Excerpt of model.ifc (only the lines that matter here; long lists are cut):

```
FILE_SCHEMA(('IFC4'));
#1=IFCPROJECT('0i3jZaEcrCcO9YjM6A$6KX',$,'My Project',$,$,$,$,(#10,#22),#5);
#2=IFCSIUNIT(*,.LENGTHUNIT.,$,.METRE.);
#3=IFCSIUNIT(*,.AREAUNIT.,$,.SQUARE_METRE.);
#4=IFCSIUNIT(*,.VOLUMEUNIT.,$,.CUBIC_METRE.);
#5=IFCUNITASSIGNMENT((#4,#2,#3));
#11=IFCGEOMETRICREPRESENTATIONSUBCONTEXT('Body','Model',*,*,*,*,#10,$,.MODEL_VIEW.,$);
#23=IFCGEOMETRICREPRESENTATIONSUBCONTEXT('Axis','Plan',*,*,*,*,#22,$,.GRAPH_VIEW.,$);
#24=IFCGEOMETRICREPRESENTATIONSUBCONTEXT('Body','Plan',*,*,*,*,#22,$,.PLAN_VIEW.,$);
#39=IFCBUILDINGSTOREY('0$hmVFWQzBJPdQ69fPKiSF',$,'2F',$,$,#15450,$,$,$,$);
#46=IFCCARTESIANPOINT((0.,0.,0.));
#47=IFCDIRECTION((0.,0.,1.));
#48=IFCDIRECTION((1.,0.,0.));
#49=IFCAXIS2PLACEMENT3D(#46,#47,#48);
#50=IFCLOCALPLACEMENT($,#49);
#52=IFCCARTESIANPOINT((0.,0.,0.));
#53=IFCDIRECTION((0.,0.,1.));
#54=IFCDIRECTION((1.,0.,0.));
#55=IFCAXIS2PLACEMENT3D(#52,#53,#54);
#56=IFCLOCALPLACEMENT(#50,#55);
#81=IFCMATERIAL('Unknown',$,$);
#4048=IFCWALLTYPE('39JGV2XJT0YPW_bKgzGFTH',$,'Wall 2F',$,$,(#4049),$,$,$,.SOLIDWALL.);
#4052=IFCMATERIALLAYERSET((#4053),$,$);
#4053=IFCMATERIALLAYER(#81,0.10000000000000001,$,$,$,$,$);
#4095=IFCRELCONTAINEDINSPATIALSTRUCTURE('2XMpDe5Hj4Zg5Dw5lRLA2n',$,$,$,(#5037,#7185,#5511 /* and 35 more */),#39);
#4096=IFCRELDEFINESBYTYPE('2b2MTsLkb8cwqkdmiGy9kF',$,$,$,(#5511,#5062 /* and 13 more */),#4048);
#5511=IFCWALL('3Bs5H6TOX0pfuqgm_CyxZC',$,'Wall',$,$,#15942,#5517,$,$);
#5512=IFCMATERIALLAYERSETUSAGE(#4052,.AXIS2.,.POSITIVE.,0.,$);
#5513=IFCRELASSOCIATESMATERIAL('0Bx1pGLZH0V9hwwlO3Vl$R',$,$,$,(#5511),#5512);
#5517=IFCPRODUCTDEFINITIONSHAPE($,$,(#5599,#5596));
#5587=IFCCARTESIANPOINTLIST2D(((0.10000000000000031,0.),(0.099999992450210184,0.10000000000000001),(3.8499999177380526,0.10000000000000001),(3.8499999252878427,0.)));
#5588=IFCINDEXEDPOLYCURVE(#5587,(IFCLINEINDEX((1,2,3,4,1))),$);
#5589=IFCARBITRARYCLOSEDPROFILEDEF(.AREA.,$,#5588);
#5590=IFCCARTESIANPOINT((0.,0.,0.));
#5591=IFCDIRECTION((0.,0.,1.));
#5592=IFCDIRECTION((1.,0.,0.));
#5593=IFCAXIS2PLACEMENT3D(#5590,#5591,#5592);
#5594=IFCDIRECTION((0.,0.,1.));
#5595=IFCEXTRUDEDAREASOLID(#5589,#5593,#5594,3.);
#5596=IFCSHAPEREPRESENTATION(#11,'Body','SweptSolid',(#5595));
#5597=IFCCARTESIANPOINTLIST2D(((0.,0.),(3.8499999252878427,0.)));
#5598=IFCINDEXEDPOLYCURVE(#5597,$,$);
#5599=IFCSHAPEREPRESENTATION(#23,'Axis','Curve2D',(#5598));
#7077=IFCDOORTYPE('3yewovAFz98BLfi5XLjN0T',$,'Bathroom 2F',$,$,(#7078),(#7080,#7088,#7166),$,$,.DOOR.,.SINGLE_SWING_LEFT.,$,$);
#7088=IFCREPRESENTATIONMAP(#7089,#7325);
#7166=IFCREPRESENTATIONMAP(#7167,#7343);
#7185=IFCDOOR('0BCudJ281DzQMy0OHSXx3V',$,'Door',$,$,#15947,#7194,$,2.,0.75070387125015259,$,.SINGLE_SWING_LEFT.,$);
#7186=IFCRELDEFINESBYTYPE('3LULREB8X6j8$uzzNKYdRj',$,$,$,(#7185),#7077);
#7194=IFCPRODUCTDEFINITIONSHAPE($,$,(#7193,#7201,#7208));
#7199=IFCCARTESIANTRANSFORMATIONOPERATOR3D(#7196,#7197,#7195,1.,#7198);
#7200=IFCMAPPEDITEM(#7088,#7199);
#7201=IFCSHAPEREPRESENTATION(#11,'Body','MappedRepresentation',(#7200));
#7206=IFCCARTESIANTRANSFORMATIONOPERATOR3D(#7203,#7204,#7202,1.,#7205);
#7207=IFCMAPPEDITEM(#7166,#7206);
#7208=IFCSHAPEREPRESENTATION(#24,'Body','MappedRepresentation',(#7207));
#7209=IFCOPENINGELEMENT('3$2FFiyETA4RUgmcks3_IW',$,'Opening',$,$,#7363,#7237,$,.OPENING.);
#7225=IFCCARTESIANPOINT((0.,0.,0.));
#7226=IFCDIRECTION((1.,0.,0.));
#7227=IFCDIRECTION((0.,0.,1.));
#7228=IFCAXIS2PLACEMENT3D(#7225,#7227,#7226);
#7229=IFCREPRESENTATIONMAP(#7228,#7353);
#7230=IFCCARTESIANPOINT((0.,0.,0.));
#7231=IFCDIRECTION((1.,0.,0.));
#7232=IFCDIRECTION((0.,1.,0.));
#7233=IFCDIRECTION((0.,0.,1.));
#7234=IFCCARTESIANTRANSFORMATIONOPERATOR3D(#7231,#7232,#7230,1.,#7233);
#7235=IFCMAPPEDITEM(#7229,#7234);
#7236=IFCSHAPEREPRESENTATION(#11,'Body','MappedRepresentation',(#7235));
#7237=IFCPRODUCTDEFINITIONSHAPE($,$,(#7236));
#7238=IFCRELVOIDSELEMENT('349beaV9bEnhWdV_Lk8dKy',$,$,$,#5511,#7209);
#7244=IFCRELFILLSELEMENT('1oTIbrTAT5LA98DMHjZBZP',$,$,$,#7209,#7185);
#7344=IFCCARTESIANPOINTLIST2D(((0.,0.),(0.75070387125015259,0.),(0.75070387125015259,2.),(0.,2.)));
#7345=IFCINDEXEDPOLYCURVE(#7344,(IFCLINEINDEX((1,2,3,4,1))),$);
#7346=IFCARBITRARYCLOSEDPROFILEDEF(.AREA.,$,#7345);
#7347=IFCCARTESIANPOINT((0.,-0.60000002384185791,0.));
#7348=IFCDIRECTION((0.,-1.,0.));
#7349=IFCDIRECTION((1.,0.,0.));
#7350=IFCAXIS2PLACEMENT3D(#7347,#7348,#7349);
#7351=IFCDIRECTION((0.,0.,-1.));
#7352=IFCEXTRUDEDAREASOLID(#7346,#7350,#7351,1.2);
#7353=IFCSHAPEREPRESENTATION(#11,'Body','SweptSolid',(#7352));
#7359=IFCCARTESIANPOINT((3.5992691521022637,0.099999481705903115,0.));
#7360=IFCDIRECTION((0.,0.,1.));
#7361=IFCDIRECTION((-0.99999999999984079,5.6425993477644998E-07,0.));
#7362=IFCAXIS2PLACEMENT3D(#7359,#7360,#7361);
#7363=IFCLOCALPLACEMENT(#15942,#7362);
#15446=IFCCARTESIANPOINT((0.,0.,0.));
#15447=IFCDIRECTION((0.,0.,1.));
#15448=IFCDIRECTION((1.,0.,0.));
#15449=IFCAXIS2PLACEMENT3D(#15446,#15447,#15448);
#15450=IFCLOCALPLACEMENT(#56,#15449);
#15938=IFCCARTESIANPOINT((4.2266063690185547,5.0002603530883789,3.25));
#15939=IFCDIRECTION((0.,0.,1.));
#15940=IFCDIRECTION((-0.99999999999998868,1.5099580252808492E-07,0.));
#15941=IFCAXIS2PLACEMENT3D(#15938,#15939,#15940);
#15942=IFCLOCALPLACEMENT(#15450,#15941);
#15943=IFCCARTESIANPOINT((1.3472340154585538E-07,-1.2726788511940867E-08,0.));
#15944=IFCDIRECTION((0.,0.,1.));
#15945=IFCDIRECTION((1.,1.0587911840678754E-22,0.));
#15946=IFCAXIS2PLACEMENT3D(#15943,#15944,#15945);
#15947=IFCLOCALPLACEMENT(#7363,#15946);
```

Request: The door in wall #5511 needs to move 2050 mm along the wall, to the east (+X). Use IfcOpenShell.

```python
import ifcopenshell
import ifcopenshell.api.geometry
import ifcopenshell.util.placement
import ifcopenshell.util.unit

model = ifcopenshell.open("model.ifc")
unit_scale = ifcopenshell.util.unit.calculate_unit_scale(model)

door = model.by_id(7185)
opening = door.FillsVoids[0].RelatingOpeningElement
wall = opening.VoidsElements[0].RelatingBuildingElement

wall_matrix = ifcopenshell.util.placement.get_local_placement(wall.ObjectPlacement)
shift = wall_matrix[:3, 0] * -2.05 / unit_scale
before = ifcopenshell.util.placement.get_local_placement(door.ObjectPlacement)[:3, 3].copy()

# The door is placed relative to its opening, so it follows when the opening moves.
matrix = ifcopenshell.util.placement.get_local_placement(opening.ObjectPlacement)
matrix[:3, 3] += shift
ifcopenshell.api.geometry.edit_object_placement(
    model, product=opening, matrix=matrix, is_si=False, should_transform_children=True
)

after = ifcopenshell.util.placement.get_local_placement(door.ObjectPlacement)[:3, 3]
print("door moved by", (after - before).round(3) + 0.0)

model.write("model-out.ifc")
```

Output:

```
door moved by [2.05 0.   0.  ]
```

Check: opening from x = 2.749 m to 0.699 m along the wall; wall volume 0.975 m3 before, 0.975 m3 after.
